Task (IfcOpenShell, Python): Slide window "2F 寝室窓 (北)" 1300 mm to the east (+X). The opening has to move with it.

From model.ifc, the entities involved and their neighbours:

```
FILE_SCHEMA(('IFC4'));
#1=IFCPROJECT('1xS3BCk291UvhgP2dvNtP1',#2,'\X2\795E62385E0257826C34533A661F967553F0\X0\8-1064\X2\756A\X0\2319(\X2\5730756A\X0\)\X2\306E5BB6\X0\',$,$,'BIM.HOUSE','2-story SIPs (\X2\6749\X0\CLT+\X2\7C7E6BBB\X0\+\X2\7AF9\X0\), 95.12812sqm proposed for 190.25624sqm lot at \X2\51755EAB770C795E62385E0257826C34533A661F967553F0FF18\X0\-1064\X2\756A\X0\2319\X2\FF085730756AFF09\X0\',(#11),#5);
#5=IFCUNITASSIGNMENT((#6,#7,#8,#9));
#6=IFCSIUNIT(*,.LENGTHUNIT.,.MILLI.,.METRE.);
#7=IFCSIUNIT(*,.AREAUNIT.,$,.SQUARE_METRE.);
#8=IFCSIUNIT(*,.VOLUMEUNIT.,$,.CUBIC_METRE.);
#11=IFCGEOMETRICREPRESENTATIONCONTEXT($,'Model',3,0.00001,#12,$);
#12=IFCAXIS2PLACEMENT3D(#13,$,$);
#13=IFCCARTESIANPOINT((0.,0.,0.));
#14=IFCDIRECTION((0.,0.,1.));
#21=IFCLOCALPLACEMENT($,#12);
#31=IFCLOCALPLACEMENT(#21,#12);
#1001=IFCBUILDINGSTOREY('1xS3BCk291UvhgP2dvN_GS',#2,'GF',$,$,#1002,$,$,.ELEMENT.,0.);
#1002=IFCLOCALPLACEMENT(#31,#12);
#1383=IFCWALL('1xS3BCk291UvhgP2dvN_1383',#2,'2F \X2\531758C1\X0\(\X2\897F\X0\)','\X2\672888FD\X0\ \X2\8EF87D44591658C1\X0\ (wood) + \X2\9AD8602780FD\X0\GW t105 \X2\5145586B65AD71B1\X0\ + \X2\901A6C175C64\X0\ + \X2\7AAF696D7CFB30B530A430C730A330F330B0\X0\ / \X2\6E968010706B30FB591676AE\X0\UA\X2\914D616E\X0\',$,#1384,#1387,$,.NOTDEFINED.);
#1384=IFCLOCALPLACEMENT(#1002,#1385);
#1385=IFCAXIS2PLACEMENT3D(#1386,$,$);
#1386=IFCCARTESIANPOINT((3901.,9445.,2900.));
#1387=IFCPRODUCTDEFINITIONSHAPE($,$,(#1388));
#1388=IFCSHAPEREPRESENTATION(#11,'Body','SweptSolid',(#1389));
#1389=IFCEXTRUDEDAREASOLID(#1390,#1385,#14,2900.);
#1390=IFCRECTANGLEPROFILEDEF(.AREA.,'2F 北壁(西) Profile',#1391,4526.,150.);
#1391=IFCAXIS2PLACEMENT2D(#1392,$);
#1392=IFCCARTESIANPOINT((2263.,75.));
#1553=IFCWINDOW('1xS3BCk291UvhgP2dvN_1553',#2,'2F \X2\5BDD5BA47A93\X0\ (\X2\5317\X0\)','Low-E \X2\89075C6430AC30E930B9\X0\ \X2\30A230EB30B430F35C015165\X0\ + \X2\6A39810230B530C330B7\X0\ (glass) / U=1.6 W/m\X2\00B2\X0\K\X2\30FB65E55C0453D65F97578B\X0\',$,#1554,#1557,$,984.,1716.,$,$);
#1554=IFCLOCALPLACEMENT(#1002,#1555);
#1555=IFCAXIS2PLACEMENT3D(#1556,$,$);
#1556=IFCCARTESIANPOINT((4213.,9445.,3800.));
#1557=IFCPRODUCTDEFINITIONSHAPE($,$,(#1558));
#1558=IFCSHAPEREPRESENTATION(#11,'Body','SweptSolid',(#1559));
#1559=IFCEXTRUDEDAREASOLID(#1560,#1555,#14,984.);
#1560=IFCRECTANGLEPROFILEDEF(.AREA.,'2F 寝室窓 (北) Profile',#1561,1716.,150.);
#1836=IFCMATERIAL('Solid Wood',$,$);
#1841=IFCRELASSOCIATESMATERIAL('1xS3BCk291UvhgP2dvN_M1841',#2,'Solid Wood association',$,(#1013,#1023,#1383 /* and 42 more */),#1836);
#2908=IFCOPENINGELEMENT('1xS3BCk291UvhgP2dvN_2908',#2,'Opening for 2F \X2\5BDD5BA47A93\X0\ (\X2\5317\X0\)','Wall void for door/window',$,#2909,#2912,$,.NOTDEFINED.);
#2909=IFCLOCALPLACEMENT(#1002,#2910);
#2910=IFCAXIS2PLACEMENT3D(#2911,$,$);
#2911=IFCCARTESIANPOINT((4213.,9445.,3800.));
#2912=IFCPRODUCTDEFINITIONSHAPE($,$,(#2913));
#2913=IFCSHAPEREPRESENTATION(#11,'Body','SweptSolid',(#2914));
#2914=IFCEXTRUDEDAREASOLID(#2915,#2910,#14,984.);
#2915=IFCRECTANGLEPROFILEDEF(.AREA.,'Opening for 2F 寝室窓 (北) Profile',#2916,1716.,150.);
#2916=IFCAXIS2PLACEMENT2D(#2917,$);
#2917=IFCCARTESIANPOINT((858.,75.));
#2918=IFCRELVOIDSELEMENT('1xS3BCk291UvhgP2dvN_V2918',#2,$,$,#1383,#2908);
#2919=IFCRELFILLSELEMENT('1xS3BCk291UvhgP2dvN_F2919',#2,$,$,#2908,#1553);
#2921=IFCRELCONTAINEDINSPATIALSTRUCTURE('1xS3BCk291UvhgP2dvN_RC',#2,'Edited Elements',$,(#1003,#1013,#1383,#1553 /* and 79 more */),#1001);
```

```python
import ifcopenshell
import ifcopenshell.api.geometry
import ifcopenshell.util.placement

model = ifcopenshell.open("model.ifc")

window = model.by_guid("1xS3BCk291UvhgP2dvN_1553")
opening = window.FillsVoids[0].RelatingOpeningElement
wall = opening.VoidsElements[0].RelatingBuildingElement

wall_matrix = ifcopenshell.util.placement.get_local_placement(wall.ObjectPlacement)
shift = wall_matrix[:3, 0] * 1300.0
before = ifcopenshell.util.placement.get_local_placement(window.ObjectPlacement)[:3, 3].copy()

# The window is not placed relative to its opening, so move both.
for product in (opening, window):
    matrix = ifcopenshell.util.placement.get_local_placement(product.ObjectPlacement)
    matrix[:3, 3] += shift
    ifcopenshell.api.geometry.edit_object_placement(model, product=product, matrix=matrix, is_si=False)

after = ifcopenshell.util.placement.get_local_placement(window.ObjectPlacement)[:3, 3]
print("window moved by", (after - before).round(3) + 0.0)

model.write("model-out.ifc")
```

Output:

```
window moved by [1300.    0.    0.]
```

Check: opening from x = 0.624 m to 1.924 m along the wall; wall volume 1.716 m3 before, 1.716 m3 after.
